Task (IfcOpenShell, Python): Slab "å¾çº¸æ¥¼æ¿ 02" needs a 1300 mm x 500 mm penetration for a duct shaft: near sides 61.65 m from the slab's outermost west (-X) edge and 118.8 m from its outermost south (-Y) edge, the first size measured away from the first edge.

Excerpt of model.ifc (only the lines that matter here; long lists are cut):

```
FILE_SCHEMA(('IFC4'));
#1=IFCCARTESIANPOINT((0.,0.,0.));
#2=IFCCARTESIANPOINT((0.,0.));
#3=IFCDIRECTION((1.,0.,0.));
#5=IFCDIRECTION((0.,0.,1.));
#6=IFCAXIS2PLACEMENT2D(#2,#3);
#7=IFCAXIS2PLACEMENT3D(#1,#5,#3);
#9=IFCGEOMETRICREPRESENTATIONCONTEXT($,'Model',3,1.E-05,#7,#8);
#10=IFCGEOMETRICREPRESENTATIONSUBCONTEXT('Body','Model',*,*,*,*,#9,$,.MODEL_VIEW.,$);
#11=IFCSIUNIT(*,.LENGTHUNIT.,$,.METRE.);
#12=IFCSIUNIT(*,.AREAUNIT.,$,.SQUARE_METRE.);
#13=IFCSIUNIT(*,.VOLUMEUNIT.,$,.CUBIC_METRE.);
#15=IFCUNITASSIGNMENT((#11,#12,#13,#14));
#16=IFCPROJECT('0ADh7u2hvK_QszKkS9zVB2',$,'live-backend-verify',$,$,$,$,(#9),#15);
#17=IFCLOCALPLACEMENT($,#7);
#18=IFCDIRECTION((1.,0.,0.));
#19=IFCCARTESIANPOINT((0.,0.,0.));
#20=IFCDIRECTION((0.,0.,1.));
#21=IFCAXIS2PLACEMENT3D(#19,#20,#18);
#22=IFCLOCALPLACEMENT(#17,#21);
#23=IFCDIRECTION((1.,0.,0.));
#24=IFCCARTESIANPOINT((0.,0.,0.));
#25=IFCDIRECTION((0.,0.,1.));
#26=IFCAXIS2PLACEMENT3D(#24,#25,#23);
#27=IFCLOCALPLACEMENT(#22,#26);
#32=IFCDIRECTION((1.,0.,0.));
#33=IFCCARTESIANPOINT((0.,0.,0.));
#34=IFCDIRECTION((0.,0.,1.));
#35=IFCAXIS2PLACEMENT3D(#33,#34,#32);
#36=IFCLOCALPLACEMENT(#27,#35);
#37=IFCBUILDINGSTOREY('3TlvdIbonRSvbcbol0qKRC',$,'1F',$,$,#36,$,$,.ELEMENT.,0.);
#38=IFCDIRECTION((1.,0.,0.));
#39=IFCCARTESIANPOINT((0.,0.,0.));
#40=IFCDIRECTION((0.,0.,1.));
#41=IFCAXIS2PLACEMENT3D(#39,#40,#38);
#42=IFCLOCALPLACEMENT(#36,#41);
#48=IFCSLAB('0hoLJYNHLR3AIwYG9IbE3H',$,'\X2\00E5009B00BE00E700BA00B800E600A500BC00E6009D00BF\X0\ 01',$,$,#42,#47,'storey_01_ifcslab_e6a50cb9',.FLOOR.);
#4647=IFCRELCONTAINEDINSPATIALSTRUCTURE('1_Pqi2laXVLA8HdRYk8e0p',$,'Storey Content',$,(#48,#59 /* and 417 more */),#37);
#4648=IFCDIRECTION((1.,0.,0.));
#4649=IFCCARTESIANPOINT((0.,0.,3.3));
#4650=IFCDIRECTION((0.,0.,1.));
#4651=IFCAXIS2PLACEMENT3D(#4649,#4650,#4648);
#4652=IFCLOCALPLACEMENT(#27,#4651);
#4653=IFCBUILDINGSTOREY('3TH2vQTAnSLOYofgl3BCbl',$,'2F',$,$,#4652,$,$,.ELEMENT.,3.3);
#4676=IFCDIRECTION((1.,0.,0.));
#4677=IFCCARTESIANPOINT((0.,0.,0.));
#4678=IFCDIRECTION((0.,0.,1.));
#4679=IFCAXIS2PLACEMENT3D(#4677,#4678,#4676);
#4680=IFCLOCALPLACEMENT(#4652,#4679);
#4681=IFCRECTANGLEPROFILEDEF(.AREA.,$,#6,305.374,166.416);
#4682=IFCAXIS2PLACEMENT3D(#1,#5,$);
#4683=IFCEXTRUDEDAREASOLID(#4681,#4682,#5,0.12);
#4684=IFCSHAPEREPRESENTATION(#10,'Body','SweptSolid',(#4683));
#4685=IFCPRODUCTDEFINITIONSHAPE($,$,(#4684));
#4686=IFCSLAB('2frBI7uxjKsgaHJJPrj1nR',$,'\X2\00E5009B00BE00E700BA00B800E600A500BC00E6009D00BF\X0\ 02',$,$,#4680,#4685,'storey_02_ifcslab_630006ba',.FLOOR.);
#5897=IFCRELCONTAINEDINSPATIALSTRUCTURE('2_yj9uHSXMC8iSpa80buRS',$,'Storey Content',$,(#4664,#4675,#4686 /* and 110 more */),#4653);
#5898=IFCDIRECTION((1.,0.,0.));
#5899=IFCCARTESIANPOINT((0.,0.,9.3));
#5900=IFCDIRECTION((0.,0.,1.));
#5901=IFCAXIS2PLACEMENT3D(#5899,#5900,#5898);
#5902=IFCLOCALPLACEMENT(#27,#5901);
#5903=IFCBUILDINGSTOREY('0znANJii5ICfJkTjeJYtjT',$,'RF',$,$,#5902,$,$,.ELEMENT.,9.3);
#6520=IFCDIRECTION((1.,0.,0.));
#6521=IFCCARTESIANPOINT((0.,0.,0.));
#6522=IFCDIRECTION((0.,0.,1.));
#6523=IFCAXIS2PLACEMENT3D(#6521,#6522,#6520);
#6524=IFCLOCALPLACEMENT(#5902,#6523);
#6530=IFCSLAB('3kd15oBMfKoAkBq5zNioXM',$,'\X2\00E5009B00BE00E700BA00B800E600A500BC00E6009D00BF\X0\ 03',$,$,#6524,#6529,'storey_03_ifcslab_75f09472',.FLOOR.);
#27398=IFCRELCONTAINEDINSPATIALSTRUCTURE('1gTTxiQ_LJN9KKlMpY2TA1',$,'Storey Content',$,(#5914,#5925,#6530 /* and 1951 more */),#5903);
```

```python
import numpy as np
import ifcopenshell
import ifcopenshell.api.feature
import ifcopenshell.api.geometry
import ifcopenshell.api.root
import ifcopenshell.geom
import ifcopenshell.util.placement
import ifcopenshell.util.representation
import ifcopenshell.util.shape
import ifcopenshell.util.unit

model = ifcopenshell.open("model.ifc")
unit_scale = ifcopenshell.util.unit.calculate_unit_scale(model)
settings = ifcopenshell.geom.settings()


def volume(element):
    """Net volume in cubic metres, openings subtracted."""
    shape = ifcopenshell.geom.create_shape(settings, element)
    return ifcopenshell.util.shape.get_volume(shape.geometry)


slab = model.by_guid("2frBI7uxjKsgaHJJPrj1nR")
before = volume(slab)

# Extent in the slab's own axes, in metres. The edges named are its -X and -Y sides.
slab_shape = ifcopenshell.geom.create_shape(settings, slab)
vertices = ifcopenshell.util.shape.get_vertices(slab_shape.geometry)
x_min, y_min, bottom = vertices.min(axis=0)
top = vertices[:, 2].max()

opening = ifcopenshell.api.root.create_entity(model, ifc_class="IfcOpeningElement", name="Duct shaft opening", predefined_type="OPENING")
context = ifcopenshell.util.representation.get_context(model, "Model", "Body", "MODEL_VIEW")
width, depth = 1.3, 0.5
outline = [(0.0, 0.0), (width, 0.0), (width, depth), (0.0, depth), (0.0, 0.0)]
# Overshoot both faces by 50 mm so the cut is clean.
shape = ifcopenshell.api.geometry.add_slab_representation(
    model, context=context, depth=top - bottom + 0.1, polyline=outline
)
ifcopenshell.api.geometry.assign_representation(model, product=opening, representation=shape)

matrix = ifcopenshell.util.placement.get_local_placement(slab.ObjectPlacement)
matrix[:, 3] = matrix @ np.append(np.array([x_min + 61.65, y_min + 118.8, bottom - 0.05]) / unit_scale, 1.0)
ifcopenshell.api.geometry.edit_object_placement(model, product=opening, matrix=matrix, is_si=False)
ifcopenshell.api.feature.add_feature(model, feature=opening, element=slab)

after = volume(slab)

print(f"slab volume {before:.3f} -> {after:.3f} m3")

model.write("model_edited.ifc")
```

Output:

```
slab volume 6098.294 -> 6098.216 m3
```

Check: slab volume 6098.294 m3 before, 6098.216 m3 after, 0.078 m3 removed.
